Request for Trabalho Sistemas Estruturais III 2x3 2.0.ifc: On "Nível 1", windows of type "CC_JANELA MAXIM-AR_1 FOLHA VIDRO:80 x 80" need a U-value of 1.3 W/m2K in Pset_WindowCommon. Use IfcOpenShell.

First a look at what the model holds.

```python
import ifcopenshell
import ifcopenshell.util.element

model = ifcopenshell.open("Trabalho Sistemas Estruturais III 2x3 2.0.ifc")
print(model.schema)
storey = next(s for s in model.by_type("IfcBuildingStorey") if s.Name == "Nível 1")
windows = [e for e in ifcopenshell.util.element.get_decomposition(storey) if e.is_a("IfcWindow")]
seen = {}
for e in windows:
    element_type = ifcopenshell.util.element.get_type(e)
    key = (element_type.Name if element_type != e and element_type else None, ifcopenshell.util.element.get_pset(e, "Pset_WindowCommon", "ThermalTransmittance"))
    seen[key] = seen.get(key, 0) + 1
for (name, value), count in sorted(seen.items(), key=str):
    print(count, "x", name, "|", value)
```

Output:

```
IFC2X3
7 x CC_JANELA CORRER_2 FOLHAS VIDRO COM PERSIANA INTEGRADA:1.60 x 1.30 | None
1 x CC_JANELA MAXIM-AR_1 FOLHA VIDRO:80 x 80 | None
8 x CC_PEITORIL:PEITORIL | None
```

```python
import ifcopenshell
import ifcopenshell.api.pset
import ifcopenshell.util.element

model = ifcopenshell.open("Trabalho Sistemas Estruturais III 2x3 2.0.ifc")

storey = next(s for s in model.by_type("IfcBuildingStorey") if s.Name == "Nível 1")
windows = [e for e in ifcopenshell.util.element.get_decomposition(storey) if e.is_a("IfcWindow")]

count = 0
for e in windows:
    element_type = ifcopenshell.util.element.get_type(e)
    if element_type in (None, e) or element_type.Name != "CC_JANELA MAXIM-AR_1 FOLHA VIDRO:80 x 80":
        continue
    # add_pset returns the element's existing set when there is one.
    pset = ifcopenshell.api.pset.add_pset(model, product=e, name="Pset_WindowCommon")
    ifcopenshell.api.pset.edit_pset(model, pset=pset, properties={"ThermalTransmittance": 1.3})
    count += 1

print(count, "windows updated")

model.write("Trabalho Sistemas Estruturais III 2x3 2.0_updated.ifc")
```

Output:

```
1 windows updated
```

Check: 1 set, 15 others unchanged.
